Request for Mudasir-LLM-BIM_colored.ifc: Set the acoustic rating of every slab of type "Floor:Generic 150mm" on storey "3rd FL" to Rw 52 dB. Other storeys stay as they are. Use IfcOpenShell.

First a look at what the model holds.

```python
import ifcopenshell
import ifcopenshell.util.element

model = ifcopenshell.open("Mudasir-LLM-BIM_colored.ifc")
print(model.schema)
storey = next(s for s in model.by_type("IfcBuildingStorey") if s.Name == "3rd FL")
slabs = [e for e in ifcopenshell.util.element.get_decomposition(storey) if e.is_a("IfcSlab")]
seen = {}
for e in slabs:
    element_type = ifcopenshell.util.element.get_type(e)
    key = (element_type.Name if element_type != e and element_type else None, ifcopenshell.util.element.get_pset(e, "Pset_SlabCommon", "AcousticRating"))
    seen[key] = seen.get(key, 0) + 1
for (name, value), count in sorted(seen.items(), key=str):
    print(count, "x", name, "|", value)
```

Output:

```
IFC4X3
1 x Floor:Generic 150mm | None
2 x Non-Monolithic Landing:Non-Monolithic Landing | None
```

```python
import ifcopenshell
import ifcopenshell.api.pset
import ifcopenshell.util.element

model = ifcopenshell.open("Mudasir-LLM-BIM_colored.ifc")

storey = next(s for s in model.by_type("IfcBuildingStorey") if s.Name == "3rd FL")
slabs = [e for e in ifcopenshell.util.element.get_decomposition(storey) if e.is_a("IfcSlab")]

count = 0
for e in slabs:
    element_type = ifcopenshell.util.element.get_type(e)
    if element_type in (None, e) or element_type.Name != "Floor:Generic 150mm":
        continue
    # add_pset returns the element's existing set when there is one.
    pset = ifcopenshell.api.pset.add_pset(model, product=e, name="Pset_SlabCommon")
    ifcopenshell.api.pset.edit_pset(model, pset=pset, properties={"AcousticRating": "Rw 52 dB"})
    count += 1

print(count, "slabs updated")

model.write("Mudasir-LLM-BIM_colored_edited.ifc")
```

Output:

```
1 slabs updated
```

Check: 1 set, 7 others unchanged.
